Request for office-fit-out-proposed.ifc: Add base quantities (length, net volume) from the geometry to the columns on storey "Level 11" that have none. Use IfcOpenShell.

First a look at what the model holds.

```python
import ifcopenshell
import ifcopenshell.util.element
import ifcopenshell.util.unit

model = ifcopenshell.open("office-fit-out-proposed.ifc")
print(model.schema)
for unit_type in ("LENGTHUNIT", "AREAUNIT", "VOLUMEUNIT"):
    print(unit_type, ifcopenshell.util.unit.calculate_unit_scale(model, unit_type))
storey = next(s for s in model.by_type("IfcBuildingStorey") if s.Name == "Level 11")
columns = [e for e in ifcopenshell.util.element.get_decomposition(storey) if e.is_a("IfcColumn")]
for e in sorted(columns, key=lambda e: e.id()):
    print(e.id(), e.is_a(), e.Name, list(ifcopenshell.util.element.get_psets(e, qtos_only=True)), sep=" | ")
```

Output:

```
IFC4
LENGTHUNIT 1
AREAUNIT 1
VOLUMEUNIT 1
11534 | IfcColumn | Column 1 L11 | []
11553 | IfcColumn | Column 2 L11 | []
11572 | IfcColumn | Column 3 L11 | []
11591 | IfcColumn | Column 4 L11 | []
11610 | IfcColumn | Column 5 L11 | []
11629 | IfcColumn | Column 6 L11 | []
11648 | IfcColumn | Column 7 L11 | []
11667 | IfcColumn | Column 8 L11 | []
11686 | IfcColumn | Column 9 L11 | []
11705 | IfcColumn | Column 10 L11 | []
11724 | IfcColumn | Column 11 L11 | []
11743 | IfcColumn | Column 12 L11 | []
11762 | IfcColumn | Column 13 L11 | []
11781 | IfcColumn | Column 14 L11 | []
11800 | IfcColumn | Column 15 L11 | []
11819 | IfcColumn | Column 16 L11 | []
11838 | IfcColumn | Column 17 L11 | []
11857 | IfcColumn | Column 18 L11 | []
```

```python
import ifcopenshell
import ifcopenshell.api.pset
import ifcopenshell.geom
import ifcopenshell.util.element
import ifcopenshell.util.shape
import ifcopenshell.util.unit

model = ifcopenshell.open("office-fit-out-proposed.ifc")
unit_scale = ifcopenshell.util.unit.calculate_unit_scale(model)
volume_scale = ifcopenshell.util.unit.calculate_unit_scale(model, "VOLUMEUNIT")
settings = ifcopenshell.geom.settings()

storey = next(s for s in model.by_type("IfcBuildingStorey") if s.Name == "Level 11")
columns = [e for e in ifcopenshell.util.element.get_decomposition(storey) if e.is_a("IfcColumn")]

for e in sorted(columns, key=lambda e: e.id()):
    if ifcopenshell.util.element.get_psets(e, qtos_only=True, should_inherit=False):
        continue
    # Geometry comes back in metres, in the element's own axes.
    shape = ifcopenshell.geom.create_shape(settings, e)
    values = {
        "Length": ifcopenshell.util.shape.get_z(shape.geometry) / unit_scale,
        "NetVolume": ifcopenshell.util.shape.get_volume(shape.geometry) / volume_scale,
    }
    qto = ifcopenshell.api.pset.add_qto(model, product=e, name="Qto_ColumnBaseQuantities")
    ifcopenshell.api.pset.edit_qto(model, qto=qto, properties=values)
    print(e.id(), {k: round(v, 3) for k, v in values.items()})

model.write("office-fit-out-proposed_rev.ifc")
```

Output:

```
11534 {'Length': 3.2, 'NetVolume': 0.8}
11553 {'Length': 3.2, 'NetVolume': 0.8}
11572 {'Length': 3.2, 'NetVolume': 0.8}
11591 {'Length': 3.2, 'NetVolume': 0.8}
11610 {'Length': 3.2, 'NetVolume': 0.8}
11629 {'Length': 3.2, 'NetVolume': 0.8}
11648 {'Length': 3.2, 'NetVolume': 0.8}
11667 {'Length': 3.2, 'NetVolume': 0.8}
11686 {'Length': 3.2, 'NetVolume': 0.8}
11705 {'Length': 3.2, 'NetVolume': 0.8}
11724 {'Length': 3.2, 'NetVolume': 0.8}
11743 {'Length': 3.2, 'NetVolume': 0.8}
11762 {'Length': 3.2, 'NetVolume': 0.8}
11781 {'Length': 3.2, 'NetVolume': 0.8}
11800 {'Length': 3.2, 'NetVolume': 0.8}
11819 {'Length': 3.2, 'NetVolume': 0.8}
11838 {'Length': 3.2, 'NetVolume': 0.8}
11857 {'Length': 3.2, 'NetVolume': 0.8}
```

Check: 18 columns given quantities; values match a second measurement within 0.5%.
